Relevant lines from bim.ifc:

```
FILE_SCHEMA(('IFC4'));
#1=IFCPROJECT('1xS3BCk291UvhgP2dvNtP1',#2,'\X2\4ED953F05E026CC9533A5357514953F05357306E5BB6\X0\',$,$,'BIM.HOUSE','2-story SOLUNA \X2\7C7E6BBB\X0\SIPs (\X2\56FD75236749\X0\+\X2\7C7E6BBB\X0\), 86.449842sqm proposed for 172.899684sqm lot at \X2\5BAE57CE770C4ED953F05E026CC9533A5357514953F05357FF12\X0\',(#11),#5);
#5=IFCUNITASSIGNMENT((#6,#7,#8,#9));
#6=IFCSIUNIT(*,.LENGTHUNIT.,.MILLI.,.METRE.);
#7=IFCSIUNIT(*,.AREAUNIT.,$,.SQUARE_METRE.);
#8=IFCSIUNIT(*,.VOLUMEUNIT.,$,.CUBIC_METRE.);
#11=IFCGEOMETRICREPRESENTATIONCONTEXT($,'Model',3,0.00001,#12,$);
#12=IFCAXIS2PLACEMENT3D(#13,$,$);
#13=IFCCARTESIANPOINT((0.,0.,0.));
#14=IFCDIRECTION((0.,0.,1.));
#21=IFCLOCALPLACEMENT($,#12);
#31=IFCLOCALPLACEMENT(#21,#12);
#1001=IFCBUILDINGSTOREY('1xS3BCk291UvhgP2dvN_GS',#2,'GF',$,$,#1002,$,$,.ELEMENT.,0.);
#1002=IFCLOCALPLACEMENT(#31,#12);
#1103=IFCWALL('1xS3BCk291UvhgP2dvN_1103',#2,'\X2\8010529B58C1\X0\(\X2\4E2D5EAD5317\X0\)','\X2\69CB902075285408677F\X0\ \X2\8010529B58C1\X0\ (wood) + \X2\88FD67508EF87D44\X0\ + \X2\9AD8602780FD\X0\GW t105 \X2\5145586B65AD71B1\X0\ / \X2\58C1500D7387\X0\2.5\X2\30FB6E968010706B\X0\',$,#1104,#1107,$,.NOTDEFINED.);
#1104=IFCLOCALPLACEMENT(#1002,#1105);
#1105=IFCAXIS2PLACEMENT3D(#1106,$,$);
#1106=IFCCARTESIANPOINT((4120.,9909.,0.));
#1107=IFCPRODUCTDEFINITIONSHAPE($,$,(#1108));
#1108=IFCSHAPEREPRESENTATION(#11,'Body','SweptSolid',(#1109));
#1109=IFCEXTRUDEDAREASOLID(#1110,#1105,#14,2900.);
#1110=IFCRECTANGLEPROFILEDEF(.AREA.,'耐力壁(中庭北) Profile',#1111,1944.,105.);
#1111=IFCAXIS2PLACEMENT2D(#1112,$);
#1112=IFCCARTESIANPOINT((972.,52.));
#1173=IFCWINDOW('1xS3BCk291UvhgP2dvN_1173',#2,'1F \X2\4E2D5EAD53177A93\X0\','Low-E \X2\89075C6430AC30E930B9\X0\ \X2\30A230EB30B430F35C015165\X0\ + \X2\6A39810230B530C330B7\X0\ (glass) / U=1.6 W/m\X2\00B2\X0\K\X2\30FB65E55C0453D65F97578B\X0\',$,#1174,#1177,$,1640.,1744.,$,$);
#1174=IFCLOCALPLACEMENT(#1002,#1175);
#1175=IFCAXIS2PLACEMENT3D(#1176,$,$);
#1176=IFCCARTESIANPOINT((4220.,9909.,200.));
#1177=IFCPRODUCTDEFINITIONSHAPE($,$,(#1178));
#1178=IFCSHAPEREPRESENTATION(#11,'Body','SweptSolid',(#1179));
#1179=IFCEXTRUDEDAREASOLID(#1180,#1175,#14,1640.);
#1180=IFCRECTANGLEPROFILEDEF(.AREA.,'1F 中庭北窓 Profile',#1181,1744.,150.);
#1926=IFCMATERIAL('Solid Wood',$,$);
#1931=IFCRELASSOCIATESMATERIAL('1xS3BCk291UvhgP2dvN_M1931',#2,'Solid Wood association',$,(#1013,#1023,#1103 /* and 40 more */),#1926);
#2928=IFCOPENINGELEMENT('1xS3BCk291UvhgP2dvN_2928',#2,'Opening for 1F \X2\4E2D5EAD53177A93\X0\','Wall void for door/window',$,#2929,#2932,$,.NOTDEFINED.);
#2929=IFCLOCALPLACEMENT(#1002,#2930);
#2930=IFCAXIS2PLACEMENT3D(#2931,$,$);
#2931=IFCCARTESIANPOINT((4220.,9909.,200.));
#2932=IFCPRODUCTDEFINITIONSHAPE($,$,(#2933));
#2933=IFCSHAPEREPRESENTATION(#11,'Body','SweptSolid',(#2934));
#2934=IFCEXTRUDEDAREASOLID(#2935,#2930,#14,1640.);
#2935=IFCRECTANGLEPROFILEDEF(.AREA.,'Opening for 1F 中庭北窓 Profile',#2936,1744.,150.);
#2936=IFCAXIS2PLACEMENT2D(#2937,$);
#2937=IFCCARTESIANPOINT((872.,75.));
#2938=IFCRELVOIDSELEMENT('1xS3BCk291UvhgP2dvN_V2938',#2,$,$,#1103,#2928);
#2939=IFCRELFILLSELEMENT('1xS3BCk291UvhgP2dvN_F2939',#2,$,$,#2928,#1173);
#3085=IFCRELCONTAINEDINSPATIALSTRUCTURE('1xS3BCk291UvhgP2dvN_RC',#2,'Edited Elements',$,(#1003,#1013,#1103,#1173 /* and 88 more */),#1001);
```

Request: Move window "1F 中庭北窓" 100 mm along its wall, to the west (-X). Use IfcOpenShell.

```python
import ifcopenshell
import ifcopenshell.api.geometry
import ifcopenshell.util.placement

model = ifcopenshell.open("bim.ifc")

window = model.by_guid("1xS3BCk291UvhgP2dvN_1173")
opening = window.FillsVoids[0].RelatingOpeningElement
wall = opening.VoidsElements[0].RelatingBuildingElement

wall_matrix = ifcopenshell.util.placement.get_local_placement(wall.ObjectPlacement)
shift = wall_matrix[:3, 0] * -100.0
before = ifcopenshell.util.placement.get_local_placement(window.ObjectPlacement)[:3, 3].copy()

# The window is not placed relative to its opening, so move both.
for product in (opening, window):
    matrix = ifcopenshell.util.placement.get_local_placement(product.ObjectPlacement)
    matrix[:3, 3] += shift
    ifcopenshell.api.geometry.edit_object_placement(model, product=product, matrix=matrix, is_si=False)

after = ifcopenshell.util.placement.get_local_placement(window.ObjectPlacement)[:3, 3]
print("window moved by", (after - before).round(3) + 0.0)

model.write("bim_edited.ifc")
```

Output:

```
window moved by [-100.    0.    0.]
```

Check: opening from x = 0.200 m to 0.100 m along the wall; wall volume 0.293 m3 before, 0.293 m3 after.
